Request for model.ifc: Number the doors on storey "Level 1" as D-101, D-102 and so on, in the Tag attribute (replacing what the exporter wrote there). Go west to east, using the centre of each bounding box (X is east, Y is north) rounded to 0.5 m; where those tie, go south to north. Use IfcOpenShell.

First a look at what the model holds.

```python
import ifcopenshell
import ifcopenshell.util.element
import ifcopenshell.util.placement

model = ifcopenshell.open("model.ifc")
print(model.schema)
storey = next(s for s in model.by_type("IfcBuildingStorey") if s.Name == "Level 1")
doors = [e for e in ifcopenshell.util.element.get_decomposition(storey) if e.is_a("IfcDoor")]
for e in sorted(doors, key=lambda e: e.id()):
    origin = ifcopenshell.util.placement.get_local_placement(e.ObjectPlacement)[:3, 3]
    print(e.id(), e.Tag, e.Name, origin.round(2) + 0.0, sep=" | ")
```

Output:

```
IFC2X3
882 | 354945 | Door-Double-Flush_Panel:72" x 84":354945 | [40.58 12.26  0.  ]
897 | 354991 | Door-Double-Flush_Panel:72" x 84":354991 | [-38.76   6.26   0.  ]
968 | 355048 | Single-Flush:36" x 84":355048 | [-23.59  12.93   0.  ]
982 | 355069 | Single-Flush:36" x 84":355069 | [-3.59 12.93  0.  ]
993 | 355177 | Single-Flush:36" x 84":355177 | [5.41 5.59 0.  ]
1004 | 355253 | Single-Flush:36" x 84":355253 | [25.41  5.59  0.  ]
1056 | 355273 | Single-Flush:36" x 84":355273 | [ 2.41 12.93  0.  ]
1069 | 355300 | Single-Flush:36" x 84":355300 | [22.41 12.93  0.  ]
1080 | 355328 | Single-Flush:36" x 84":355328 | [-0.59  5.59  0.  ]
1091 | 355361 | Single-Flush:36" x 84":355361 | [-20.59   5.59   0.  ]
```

```python
import ifcopenshell
import ifcopenshell.geom
import ifcopenshell.util.element
import ifcopenshell.util.shape

model = ifcopenshell.open("model.ifc")
settings = ifcopenshell.geom.settings()
settings.set("use-world-coords", True)


def centre(element):
    shape = ifcopenshell.geom.create_shape(settings, element)
    return ifcopenshell.util.shape.get_bbox_centroid(shape.geometry)


storey = next(s for s in model.by_type("IfcBuildingStorey") if s.Name == "Level 1")
doors = [e for e in ifcopenshell.util.element.get_decomposition(storey) if e.is_a("IfcDoor")]

# Insertion points can sit at a corner or the storey origin, so sort by the geometry (in metres).
centres = {e: centre(e) for e in doors}
doors.sort(key=lambda e: (round(centres[e][0] / 0.5), centres[e][1]))

for i, e in enumerate(doors, start=1):
    number = f"D-1{i:02d}"
    e.Tag = number
    print(e.id(), number)

model.write("model_v2.ifc")
```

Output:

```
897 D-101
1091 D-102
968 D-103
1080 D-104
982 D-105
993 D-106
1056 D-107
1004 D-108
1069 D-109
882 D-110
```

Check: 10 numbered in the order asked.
